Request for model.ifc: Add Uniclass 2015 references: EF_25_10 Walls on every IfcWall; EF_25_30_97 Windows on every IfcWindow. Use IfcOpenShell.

First a look at what the model holds.

```python
import ifcopenshell

model = ifcopenshell.open("model.ifc")
print(model.schema)
print("classifications:", [c.Name for c in model.by_type("IfcClassification")])
for ifc_class in ("IfcDoor", "IfcRoof", "IfcStair", "IfcWall", "IfcWindow"):
    print(ifc_class, len(model.by_type(ifc_class)))
```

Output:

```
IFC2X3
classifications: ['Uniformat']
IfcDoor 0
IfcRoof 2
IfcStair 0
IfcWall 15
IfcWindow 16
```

```python
import ifcopenshell
import ifcopenshell.api.classification

model = ifcopenshell.open("model.ifc")

# IFC2X3 requires Source and Edition and has no link from the project to the system.
system = model.create_entity("IfcClassification", Source="NBS", Edition="2015", Name="Uniclass 2015")

codes = {
    "IfcWall": ("EF_25_10", "Walls"),
    "IfcWindow": ("EF_25_30_97", "Windows"),
}
for ifc_class, (code, name) in codes.items():
    products = model.by_type(ifc_class)
    ifcopenshell.api.classification.add_reference(
        model, products=products, classification=system, identification=code, name=name
    )
    print(code, len(products))

model.write("model-out.ifc")
```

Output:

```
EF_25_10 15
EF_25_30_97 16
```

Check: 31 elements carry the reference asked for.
